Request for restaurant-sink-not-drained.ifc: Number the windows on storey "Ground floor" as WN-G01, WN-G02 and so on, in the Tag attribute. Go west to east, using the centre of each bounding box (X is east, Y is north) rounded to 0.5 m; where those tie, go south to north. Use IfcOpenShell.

First a look at what the model holds.

```python
import ifcopenshell
import ifcopenshell.util.element
import ifcopenshell.util.placement

model = ifcopenshell.open("restaurant-sink-not-drained.ifc")
print(model.schema)
storey = next(s for s in model.by_type("IfcBuildingStorey") if s.Name == "Ground floor")
windows = [e for e in ifcopenshell.util.element.get_decomposition(storey) if e.is_a("IfcWindow")]
for e in sorted(windows, key=lambda e: e.id()):
    origin = ifcopenshell.util.placement.get_local_placement(e.ObjectPlacement)[:3, 3]
    print(e.id(), e.Tag, e.Name, origin.round(2) + 0.0, sep=" | ")
```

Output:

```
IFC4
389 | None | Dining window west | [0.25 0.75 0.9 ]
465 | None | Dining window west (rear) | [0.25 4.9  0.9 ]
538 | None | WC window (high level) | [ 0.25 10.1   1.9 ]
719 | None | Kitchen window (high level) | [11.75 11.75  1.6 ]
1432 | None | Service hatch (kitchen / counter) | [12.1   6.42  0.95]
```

```python
import ifcopenshell
import ifcopenshell.geom
import ifcopenshell.util.element
import ifcopenshell.util.shape

model = ifcopenshell.open("restaurant-sink-not-drained.ifc")
settings = ifcopenshell.geom.settings()
settings.set("use-world-coords", True)


def centre(element):
    shape = ifcopenshell.geom.create_shape(settings, element)
    return ifcopenshell.util.shape.get_bbox_centroid(shape.geometry)


storey = next(s for s in model.by_type("IfcBuildingStorey") if s.Name == "Ground floor")
windows = [e for e in ifcopenshell.util.element.get_decomposition(storey) if e.is_a("IfcWindow")]

# Insertion points can sit at a corner or the storey origin, so sort by the geometry (in metres).
centres = {e: centre(e) for e in windows}
windows.sort(key=lambda e: (round(centres[e][0] / 0.5), centres[e][1]))

for i, e in enumerate(windows, start=1):
    number = f"WN-G{i:02d}"
    e.Tag = number
    print(e.id(), number)

model.write("restaurant-sink-not-drained_v2.ifc")
```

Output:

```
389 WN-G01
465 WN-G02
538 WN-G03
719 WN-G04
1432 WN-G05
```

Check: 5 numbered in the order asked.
